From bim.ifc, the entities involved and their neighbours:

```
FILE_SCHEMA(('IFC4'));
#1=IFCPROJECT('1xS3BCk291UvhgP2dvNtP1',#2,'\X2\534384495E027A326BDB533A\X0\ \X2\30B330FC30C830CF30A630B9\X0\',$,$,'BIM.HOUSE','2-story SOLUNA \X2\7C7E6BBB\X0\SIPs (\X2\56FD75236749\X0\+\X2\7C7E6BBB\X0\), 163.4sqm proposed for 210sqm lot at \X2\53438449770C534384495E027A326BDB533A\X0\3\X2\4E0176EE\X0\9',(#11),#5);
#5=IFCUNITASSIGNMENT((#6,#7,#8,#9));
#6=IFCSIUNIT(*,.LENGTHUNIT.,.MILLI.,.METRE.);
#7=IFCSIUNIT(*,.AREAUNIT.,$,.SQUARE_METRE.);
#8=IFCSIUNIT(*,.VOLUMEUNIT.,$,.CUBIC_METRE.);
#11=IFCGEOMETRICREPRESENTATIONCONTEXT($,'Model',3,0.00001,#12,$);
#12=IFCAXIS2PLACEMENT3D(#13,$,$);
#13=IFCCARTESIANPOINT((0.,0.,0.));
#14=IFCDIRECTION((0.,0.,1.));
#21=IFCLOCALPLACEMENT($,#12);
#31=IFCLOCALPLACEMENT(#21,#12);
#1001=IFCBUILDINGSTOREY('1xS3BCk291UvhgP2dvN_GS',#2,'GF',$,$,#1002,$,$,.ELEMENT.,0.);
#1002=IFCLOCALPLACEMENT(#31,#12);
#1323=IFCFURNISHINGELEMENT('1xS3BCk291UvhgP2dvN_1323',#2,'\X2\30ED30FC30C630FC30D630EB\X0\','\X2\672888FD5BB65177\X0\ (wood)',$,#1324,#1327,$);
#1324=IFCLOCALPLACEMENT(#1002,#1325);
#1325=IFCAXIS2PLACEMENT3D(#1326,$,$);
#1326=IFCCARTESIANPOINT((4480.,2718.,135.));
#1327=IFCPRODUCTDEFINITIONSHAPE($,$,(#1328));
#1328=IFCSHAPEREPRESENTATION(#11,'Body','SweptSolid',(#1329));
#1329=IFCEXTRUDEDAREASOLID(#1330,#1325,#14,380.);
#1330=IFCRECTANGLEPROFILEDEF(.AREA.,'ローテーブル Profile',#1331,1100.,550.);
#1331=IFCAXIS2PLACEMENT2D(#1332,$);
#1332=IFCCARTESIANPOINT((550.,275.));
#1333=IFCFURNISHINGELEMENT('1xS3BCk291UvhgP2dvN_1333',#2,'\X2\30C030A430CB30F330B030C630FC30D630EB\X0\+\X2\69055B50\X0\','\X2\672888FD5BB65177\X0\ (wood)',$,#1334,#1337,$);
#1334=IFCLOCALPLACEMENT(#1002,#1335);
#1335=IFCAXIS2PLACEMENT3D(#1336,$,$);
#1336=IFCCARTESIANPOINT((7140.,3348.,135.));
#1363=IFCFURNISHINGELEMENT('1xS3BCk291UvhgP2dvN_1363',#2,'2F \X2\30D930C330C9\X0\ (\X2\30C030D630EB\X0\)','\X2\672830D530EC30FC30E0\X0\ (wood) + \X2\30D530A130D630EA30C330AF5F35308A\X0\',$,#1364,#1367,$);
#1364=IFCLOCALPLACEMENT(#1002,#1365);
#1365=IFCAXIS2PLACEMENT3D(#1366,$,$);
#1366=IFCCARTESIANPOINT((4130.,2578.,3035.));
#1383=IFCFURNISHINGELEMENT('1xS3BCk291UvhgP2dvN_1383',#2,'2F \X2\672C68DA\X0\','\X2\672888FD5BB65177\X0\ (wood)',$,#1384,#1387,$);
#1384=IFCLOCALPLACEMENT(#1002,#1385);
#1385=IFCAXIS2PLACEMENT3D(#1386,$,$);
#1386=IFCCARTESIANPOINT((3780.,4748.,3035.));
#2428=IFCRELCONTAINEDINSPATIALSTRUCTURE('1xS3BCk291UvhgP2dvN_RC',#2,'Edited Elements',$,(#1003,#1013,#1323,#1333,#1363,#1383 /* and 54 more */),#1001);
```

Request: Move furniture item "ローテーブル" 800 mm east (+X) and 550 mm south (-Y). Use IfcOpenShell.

```python
import ifcopenshell
import ifcopenshell.api.geometry
import ifcopenshell.util.placement

model = ifcopenshell.open("bim.ifc")

item = model.by_guid("1xS3BCk291UvhgP2dvN_1323")
matrix = ifcopenshell.util.placement.get_local_placement(item.ObjectPlacement)
matrix[0, 3] += 800.0
matrix[1, 3] -= 550.0
ifcopenshell.api.geometry.edit_object_placement(model, product=item, matrix=matrix, is_si=False)

print(ifcopenshell.util.placement.get_local_placement(item.ObjectPlacement).round(3) + 0.0)

model.write("bim_rev.ifc")
```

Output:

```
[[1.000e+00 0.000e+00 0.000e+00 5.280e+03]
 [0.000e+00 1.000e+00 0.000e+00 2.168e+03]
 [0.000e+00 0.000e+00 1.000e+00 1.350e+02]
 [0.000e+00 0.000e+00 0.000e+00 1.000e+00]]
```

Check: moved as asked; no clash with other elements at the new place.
